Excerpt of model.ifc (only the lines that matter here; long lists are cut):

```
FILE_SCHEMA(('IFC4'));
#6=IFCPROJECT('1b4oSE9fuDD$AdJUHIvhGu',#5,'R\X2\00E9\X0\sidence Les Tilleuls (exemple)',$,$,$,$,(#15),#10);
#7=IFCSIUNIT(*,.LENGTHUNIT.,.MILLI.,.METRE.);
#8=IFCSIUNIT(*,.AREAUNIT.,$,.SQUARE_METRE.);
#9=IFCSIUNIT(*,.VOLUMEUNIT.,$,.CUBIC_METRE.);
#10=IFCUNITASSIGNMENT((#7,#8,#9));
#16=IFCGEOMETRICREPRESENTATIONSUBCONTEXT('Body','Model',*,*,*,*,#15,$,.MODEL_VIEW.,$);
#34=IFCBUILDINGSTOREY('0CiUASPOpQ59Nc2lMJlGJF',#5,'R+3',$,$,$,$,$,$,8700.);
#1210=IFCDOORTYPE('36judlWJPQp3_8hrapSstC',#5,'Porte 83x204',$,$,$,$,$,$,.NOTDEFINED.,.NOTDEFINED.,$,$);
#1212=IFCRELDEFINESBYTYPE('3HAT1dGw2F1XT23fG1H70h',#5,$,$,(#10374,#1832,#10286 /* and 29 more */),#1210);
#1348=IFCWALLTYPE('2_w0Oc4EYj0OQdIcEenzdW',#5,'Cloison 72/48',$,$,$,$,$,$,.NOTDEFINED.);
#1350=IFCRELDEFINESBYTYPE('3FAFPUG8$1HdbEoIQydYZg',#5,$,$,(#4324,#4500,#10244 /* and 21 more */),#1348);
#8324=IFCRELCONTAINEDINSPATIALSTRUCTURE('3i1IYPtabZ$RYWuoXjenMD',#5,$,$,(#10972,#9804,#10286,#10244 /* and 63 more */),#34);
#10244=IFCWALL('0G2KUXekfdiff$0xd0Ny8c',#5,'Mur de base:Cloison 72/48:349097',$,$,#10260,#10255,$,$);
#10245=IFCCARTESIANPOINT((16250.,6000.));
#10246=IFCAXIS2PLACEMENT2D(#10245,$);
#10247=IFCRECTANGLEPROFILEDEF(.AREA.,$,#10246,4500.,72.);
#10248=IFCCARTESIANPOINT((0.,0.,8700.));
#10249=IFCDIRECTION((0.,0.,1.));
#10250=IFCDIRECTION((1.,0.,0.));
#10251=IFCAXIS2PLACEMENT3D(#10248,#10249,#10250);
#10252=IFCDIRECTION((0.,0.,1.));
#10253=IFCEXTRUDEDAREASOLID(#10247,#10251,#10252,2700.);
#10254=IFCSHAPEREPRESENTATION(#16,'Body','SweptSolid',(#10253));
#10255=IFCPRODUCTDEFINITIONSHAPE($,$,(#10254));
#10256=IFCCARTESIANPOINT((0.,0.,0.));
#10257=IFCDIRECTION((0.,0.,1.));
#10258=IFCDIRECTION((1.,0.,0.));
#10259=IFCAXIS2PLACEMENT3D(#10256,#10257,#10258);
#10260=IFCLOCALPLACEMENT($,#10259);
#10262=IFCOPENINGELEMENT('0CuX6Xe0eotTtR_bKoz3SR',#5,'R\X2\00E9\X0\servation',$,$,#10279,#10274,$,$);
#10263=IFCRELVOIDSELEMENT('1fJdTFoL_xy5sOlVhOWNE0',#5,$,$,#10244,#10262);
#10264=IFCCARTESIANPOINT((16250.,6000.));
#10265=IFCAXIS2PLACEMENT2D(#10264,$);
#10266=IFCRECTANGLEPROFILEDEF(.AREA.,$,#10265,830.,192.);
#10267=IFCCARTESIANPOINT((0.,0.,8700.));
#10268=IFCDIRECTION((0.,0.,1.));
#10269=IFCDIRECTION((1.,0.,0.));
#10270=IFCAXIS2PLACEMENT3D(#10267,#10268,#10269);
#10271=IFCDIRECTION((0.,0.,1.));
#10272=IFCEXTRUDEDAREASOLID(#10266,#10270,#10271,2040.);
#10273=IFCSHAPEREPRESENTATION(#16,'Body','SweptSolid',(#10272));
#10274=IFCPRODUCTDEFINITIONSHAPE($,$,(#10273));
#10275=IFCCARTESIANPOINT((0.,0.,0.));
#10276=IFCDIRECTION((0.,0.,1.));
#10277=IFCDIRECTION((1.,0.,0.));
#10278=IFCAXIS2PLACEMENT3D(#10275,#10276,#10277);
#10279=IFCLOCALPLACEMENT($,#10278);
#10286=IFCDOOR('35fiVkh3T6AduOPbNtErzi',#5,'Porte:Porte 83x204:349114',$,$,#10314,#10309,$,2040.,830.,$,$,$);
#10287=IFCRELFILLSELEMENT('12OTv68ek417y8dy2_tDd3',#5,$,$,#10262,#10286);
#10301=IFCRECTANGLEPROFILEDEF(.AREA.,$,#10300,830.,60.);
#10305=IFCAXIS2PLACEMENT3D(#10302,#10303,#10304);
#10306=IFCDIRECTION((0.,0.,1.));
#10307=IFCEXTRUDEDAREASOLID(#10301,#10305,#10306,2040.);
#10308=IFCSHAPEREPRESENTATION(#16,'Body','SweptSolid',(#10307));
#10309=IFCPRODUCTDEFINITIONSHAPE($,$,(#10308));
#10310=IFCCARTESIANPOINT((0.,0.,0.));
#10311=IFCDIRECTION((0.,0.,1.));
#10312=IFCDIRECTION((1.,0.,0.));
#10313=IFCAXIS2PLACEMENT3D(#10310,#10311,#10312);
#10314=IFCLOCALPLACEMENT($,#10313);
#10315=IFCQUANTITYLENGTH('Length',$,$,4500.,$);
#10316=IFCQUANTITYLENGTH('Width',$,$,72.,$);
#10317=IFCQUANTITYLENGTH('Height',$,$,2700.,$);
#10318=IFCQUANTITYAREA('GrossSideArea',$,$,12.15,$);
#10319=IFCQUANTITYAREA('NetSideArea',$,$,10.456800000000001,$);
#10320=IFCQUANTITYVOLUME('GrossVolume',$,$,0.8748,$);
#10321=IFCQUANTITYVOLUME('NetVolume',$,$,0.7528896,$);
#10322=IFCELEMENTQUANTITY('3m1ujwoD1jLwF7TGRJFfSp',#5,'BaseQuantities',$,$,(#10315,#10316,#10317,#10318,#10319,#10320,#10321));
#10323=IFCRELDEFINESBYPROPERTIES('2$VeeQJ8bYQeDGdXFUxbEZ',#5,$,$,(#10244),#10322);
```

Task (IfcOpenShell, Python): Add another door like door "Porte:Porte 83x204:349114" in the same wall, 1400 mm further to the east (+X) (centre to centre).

```python
import ifcopenshell
import ifcopenshell.api.feature
import ifcopenshell.api.geometry
import ifcopenshell.api.pset
import ifcopenshell.api.root
import ifcopenshell.geom
import ifcopenshell.util.element
import ifcopenshell.util.placement
import ifcopenshell.util.shape
import ifcopenshell.util.unit

model = ifcopenshell.open("model.ifc")
unit_scale = ifcopenshell.util.unit.calculate_unit_scale(model)
area_scale = ifcopenshell.util.unit.calculate_unit_scale(model, "AREAUNIT")
volume_scale = ifcopenshell.util.unit.calculate_unit_scale(model, "VOLUMEUNIT")
settings = ifcopenshell.geom.settings()


def volume(element):
    """Net volume in cubic metres, openings subtracted."""
    shape = ifcopenshell.geom.create_shape(settings, element)
    return ifcopenshell.util.shape.get_volume(shape.geometry)


def reuse_history(source, copy):
    """copy_class also copies each property set's owner history, people and application; keep the originals."""
    for rel in copy.IsDefinedBy:
        if rel.is_a("IfcRelDefinesByProperties") and (history := rel.RelatingPropertyDefinition.OwnerHistory):
            rel.RelatingPropertyDefinition.OwnerHistory = source.OwnerHistory
            ifcopenshell.util.element.remove_deep2(model, history)


door = model.by_guid("35fiVkh3T6AduOPbNtErzi")
opening = door.FillsVoids[0].RelatingOpeningElement
wall = opening.VoidsElements[0].RelatingBuildingElement
before = volume(wall)
shift = ifcopenshell.util.placement.get_local_placement(wall.ObjectPlacement)[:3, 0] * 1.4 / unit_scale

# copy_class copies the void relationship, type, container and properties, but no geometry.
new_opening = ifcopenshell.api.root.copy_class(model, product=opening)
new_opening.Representation = ifcopenshell.util.element.copy_deep(
    model, opening.Representation, exclude=["IfcGeometricRepresentationContext", "IfcRepresentationMap"]
)
reuse_history(opening, new_opening)
new_door = ifcopenshell.api.root.copy_class(model, product=door)
new_door.Representation = ifcopenshell.util.element.copy_deep(
    model, door.Representation, exclude=["IfcGeometricRepresentationContext", "IfcRepresentationMap"]
)
new_door.Name = "Porte:Porte 83x204"
reuse_history(door, new_door)
ifcopenshell.api.feature.add_filling(model, opening=new_opening, element=new_door)

for old, new in ((opening, new_opening), (door, new_door)):
    matrix = ifcopenshell.util.placement.get_local_placement(old.ObjectPlacement)
    matrix[:3, 3] += shift
    ifcopenshell.api.geometry.edit_object_placement(model, product=new, matrix=matrix, is_si=False)

after = volume(wall)
thickness = 0.072  # wall thickness in metres

# Update the wall's stored quantities.
qto = model.by_id(ifcopenshell.util.element.get_pset(wall, "BaseQuantities", should_inherit=False)["id"])
ifcopenshell.api.pset.edit_qto(model, qto=qto, properties={
    "NetSideArea": after / thickness / area_scale,
    "NetVolume": after / volume_scale,
})

print(f"wall volume {before:.3f} -> {after:.3f} m3")

model.write("model_edited.ifc")
```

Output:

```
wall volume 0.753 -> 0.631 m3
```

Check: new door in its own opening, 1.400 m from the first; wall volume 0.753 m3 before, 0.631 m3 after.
